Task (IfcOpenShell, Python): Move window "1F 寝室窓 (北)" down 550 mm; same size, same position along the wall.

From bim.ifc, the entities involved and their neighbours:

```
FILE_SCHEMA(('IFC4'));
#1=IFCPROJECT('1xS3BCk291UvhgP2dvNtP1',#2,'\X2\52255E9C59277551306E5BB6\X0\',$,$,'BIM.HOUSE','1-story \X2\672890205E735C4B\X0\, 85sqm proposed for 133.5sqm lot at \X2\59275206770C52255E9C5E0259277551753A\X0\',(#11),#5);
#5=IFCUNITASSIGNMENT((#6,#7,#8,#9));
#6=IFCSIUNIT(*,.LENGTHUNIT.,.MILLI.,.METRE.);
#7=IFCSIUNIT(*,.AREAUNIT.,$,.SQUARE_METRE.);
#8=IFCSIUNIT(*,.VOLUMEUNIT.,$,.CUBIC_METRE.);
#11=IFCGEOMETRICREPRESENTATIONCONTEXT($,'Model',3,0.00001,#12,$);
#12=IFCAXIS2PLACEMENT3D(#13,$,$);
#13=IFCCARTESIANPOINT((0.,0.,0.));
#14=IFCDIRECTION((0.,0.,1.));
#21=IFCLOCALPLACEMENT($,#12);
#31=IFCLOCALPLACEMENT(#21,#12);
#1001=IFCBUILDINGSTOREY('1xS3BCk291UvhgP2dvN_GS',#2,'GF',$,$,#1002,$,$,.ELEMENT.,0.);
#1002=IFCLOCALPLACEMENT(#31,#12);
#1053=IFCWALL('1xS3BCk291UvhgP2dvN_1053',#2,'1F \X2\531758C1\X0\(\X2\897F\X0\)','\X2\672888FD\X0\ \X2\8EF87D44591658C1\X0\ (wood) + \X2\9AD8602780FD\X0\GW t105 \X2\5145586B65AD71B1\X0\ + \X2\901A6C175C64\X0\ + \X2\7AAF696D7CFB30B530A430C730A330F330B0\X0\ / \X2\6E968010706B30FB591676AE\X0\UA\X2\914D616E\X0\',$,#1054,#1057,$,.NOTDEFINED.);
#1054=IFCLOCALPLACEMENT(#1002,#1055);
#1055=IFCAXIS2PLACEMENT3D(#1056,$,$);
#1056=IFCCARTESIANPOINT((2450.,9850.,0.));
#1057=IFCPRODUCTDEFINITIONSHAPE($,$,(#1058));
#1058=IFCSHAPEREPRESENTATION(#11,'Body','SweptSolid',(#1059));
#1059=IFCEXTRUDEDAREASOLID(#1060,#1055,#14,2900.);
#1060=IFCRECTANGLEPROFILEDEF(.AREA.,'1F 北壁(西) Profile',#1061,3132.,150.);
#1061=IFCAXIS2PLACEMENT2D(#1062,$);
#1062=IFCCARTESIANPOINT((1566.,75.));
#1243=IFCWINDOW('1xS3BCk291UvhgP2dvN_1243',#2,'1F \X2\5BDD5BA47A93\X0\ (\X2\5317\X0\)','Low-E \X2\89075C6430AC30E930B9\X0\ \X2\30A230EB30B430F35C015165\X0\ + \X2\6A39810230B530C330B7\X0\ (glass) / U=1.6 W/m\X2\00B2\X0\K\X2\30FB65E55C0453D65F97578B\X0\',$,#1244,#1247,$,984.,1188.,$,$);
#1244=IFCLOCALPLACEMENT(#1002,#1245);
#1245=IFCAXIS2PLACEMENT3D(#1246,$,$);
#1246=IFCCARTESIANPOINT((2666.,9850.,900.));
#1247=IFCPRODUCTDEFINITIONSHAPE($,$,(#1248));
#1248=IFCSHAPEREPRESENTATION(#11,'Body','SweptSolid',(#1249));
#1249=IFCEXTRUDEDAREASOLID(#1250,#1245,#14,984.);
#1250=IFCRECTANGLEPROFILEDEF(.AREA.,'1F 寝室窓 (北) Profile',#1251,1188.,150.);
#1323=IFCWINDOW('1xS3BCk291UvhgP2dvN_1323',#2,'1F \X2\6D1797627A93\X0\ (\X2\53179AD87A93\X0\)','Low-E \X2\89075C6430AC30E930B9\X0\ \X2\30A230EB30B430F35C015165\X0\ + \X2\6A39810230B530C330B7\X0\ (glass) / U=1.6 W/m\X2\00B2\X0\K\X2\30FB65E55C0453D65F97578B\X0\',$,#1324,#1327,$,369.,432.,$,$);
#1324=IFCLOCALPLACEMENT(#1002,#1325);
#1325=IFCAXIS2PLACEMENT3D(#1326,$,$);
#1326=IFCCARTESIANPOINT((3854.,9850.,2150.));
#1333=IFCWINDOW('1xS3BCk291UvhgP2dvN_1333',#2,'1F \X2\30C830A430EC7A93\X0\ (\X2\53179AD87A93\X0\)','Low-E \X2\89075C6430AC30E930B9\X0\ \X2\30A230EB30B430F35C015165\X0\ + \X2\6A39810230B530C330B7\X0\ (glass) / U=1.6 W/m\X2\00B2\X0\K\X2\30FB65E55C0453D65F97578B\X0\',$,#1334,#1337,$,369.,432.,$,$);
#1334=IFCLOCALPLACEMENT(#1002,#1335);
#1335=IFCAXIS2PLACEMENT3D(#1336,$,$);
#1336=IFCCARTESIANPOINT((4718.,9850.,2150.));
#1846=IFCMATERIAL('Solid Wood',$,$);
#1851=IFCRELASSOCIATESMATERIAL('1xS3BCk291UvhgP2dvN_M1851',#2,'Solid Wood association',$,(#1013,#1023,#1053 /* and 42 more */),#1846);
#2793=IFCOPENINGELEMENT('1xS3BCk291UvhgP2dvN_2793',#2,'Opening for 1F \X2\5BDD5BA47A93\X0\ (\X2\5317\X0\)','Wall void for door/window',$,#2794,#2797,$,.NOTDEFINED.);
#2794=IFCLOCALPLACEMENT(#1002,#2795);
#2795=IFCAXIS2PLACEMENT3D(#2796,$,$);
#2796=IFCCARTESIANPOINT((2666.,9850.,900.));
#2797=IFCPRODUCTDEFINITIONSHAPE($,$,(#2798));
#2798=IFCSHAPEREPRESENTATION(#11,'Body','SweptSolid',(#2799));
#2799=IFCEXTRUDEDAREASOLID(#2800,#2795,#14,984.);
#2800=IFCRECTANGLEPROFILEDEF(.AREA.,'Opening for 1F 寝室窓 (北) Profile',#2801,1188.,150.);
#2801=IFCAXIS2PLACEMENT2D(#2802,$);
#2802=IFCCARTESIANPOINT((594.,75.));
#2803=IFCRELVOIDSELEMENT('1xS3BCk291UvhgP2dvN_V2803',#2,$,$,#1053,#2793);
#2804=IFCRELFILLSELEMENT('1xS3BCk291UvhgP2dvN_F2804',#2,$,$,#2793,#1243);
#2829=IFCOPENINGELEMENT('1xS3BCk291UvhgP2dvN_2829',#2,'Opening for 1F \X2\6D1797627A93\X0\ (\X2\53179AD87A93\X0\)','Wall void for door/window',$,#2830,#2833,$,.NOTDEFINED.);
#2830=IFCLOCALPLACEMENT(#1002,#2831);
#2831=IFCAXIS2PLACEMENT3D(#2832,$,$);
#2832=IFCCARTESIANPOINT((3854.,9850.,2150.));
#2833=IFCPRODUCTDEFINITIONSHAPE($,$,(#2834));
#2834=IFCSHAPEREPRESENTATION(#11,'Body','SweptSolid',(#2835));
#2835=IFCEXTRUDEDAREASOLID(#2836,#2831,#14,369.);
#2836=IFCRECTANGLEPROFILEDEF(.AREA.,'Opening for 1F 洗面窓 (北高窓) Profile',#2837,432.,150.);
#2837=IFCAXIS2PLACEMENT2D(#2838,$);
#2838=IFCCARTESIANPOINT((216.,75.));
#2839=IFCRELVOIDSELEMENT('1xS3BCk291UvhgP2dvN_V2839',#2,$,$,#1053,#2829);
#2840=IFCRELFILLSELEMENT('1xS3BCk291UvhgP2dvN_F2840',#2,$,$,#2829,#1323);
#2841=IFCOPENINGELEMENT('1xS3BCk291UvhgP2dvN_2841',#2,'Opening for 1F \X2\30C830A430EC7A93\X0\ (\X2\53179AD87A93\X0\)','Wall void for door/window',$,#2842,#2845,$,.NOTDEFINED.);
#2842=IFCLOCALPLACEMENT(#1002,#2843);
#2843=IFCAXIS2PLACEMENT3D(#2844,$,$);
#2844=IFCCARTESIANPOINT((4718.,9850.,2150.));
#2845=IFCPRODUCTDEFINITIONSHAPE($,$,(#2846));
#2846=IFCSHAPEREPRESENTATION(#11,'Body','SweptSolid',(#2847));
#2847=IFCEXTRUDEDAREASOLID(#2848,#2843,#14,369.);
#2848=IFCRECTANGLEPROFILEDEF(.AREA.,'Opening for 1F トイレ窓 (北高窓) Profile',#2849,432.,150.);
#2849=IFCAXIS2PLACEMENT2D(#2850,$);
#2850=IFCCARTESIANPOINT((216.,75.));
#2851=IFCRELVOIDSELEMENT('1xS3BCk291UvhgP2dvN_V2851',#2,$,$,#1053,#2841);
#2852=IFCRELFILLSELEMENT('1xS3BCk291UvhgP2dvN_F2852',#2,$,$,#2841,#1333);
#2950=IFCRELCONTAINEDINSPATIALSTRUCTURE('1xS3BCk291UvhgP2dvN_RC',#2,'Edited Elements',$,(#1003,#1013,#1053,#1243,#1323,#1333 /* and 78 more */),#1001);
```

```python
import numpy as np
import ifcopenshell
import ifcopenshell.api.geometry
import ifcopenshell.util.placement
import ifcopenshell.util.unit

model = ifcopenshell.open("bim.ifc")
unit_scale = ifcopenshell.util.unit.calculate_unit_scale(model)

window = model.by_guid("1xS3BCk291UvhgP2dvN_1243")
opening = window.FillsVoids[0].RelatingOpeningElement
dz = -0.55 / unit_scale

shift = np.array([0.0, 0.0, dz])
# The window is not placed relative to its opening, so move both.
for product in (opening, window):
    matrix = ifcopenshell.util.placement.get_local_placement(product.ObjectPlacement)
    matrix[:3, 3] += shift
    ifcopenshell.api.geometry.edit_object_placement(model, product=product, matrix=matrix, is_si=False)

print(f"moved by {dz * unit_scale:+.3f} m")

model.write("bim_v2.ifc")
```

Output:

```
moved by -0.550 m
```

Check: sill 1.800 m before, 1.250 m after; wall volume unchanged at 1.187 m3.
